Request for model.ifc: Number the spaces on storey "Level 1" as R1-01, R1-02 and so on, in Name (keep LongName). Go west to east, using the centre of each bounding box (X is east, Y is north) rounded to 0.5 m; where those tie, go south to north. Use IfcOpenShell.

First a look at what the model holds.

```python
import ifcopenshell
import ifcopenshell.util.element
import ifcopenshell.util.placement

model = ifcopenshell.open("model.ifc")
print(model.schema)
storey = next(s for s in model.by_type("IfcBuildingStorey") if s.Name == "Level 1")
spaces = [e for e in ifcopenshell.util.element.get_decomposition(storey) if e.is_a("IfcSpace")]
for e in sorted(spaces, key=lambda e: e.id()):
    origin = ifcopenshell.util.placement.get_local_placement(e.ObjectPlacement)[:3, 3]
    print(e.id(), e.Name, e.LongName, origin.round(2) + 0.0, sep=" | ")
```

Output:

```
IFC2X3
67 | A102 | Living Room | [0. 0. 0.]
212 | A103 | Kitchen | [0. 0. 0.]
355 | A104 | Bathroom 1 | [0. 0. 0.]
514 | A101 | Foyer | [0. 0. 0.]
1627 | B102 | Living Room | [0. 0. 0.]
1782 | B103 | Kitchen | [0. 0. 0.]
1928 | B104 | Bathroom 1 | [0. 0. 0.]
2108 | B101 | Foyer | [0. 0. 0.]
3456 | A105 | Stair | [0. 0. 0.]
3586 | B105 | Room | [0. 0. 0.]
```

```python
import ifcopenshell
import ifcopenshell.geom
import ifcopenshell.util.element
import ifcopenshell.util.shape

model = ifcopenshell.open("model.ifc")
settings = ifcopenshell.geom.settings()
settings.set("use-world-coords", True)


def centre(element):
    shape = ifcopenshell.geom.create_shape(settings, element)
    return ifcopenshell.util.shape.get_bbox_centroid(shape.geometry)


storey = next(s for s in model.by_type("IfcBuildingStorey") if s.Name == "Level 1")
spaces = [e for e in ifcopenshell.util.element.get_decomposition(storey) if e.is_a("IfcSpace")]

# Insertion points can sit at a corner or the storey origin, so sort by the geometry (in metres).
centres = {e: centre(e) for e in spaces}
spaces.sort(key=lambda e: (round(centres[e][0] / 0.5), centres[e][1]))

for i, e in enumerate(spaces, start=1):
    number = f"R1-{i:02d}"
    e.Name = number
    print(e.id(), number)

model.write("model_v2.ifc")
```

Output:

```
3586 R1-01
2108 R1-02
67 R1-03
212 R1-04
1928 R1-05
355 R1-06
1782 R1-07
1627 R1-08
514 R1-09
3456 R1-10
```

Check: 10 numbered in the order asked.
